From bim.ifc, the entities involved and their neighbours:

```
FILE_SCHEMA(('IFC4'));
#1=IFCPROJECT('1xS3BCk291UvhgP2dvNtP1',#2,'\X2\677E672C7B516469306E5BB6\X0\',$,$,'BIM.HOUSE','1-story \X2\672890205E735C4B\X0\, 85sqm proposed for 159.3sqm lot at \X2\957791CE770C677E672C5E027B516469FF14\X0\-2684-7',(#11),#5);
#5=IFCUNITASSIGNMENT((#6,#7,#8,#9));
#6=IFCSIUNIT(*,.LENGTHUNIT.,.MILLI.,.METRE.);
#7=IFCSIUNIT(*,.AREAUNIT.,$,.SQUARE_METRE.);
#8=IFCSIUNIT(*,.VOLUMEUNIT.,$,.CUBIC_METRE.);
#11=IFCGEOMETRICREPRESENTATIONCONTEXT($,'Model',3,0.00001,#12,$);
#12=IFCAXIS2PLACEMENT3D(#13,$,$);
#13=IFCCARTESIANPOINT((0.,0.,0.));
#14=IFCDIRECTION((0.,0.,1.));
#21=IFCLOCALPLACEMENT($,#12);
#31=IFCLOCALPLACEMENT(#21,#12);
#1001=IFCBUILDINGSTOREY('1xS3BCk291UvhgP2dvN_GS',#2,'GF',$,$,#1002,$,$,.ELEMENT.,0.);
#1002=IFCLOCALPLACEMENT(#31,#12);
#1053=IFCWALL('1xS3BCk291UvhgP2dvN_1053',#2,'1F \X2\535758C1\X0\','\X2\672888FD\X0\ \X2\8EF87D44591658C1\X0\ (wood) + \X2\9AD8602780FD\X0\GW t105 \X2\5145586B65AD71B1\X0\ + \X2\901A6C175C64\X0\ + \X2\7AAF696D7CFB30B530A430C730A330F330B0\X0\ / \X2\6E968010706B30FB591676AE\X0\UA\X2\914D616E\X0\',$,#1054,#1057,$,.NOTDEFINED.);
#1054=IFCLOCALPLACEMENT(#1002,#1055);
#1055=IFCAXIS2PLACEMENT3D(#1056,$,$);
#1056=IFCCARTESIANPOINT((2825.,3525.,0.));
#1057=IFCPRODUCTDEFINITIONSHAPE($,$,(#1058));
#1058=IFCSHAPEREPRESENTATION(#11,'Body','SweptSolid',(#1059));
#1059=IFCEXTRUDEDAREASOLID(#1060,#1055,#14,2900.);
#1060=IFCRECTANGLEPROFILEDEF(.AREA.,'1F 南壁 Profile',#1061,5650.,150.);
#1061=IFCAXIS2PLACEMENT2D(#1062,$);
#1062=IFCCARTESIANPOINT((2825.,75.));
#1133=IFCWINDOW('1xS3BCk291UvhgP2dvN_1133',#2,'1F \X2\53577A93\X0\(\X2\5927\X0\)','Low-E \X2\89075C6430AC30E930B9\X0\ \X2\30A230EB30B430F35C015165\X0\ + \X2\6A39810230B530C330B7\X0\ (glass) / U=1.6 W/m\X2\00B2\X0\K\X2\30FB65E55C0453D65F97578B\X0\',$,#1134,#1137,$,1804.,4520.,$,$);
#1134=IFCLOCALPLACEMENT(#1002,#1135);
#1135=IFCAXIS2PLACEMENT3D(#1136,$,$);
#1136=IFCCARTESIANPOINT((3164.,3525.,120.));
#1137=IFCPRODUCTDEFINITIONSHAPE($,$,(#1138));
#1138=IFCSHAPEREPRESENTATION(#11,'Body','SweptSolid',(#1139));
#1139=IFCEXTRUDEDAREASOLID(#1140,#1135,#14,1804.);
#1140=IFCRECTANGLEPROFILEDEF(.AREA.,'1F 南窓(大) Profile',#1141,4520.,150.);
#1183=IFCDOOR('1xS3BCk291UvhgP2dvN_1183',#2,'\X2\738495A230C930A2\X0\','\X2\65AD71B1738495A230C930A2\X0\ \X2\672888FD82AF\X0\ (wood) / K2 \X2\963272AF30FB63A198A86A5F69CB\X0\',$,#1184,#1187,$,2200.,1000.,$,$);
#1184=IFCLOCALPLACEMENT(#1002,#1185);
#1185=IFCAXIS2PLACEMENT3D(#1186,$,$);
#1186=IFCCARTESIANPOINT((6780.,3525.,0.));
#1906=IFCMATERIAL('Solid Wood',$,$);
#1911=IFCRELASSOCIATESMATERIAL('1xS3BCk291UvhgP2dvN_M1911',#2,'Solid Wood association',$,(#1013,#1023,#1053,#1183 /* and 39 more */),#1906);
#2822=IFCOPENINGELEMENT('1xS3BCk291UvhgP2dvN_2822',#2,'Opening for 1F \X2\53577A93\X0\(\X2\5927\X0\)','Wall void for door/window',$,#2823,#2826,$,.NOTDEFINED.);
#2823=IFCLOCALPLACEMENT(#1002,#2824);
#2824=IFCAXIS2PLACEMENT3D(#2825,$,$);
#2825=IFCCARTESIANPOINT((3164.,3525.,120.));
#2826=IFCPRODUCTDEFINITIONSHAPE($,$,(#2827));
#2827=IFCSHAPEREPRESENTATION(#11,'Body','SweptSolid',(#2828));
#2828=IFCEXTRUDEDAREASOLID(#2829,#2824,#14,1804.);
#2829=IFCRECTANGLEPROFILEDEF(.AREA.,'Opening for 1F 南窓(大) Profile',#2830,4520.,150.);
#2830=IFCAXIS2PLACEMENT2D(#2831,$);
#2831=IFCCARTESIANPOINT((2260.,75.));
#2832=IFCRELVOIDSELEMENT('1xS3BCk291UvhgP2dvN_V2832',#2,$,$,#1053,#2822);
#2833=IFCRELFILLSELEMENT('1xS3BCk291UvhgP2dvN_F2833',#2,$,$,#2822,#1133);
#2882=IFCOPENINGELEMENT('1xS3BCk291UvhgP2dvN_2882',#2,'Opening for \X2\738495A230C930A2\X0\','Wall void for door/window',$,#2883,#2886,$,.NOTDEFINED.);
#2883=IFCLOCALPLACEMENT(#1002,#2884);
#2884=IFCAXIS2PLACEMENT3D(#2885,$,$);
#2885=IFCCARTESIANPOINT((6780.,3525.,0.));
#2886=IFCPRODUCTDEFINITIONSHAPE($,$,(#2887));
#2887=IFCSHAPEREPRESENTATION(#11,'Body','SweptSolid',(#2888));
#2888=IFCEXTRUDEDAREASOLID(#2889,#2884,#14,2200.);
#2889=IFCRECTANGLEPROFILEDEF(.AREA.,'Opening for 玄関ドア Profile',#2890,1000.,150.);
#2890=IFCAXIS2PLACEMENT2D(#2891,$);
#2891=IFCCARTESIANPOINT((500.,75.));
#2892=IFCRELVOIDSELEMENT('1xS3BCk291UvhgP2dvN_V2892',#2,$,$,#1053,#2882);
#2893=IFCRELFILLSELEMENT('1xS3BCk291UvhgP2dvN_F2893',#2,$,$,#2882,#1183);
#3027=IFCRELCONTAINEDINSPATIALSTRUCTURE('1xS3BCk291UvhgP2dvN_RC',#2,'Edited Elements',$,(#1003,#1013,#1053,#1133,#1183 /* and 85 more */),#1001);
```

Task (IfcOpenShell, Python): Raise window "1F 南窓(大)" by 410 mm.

```python
import numpy as np
import ifcopenshell
import ifcopenshell.api.geometry
import ifcopenshell.util.placement
import ifcopenshell.util.unit

model = ifcopenshell.open("bim.ifc")
unit_scale = ifcopenshell.util.unit.calculate_unit_scale(model)

window = model.by_id(1133)
opening = window.FillsVoids[0].RelatingOpeningElement
dz = 0.41 / unit_scale

shift = np.array([0.0, 0.0, dz])
# The window is not placed relative to its opening, so move both.
for product in (opening, window):
    matrix = ifcopenshell.util.placement.get_local_placement(product.ObjectPlacement)
    matrix[:3, 3] += shift
    ifcopenshell.api.geometry.edit_object_placement(model, product=product, matrix=matrix, is_si=False)

print(f"moved by {dz * unit_scale:+.3f} m")

model.write("bim-out.ifc")
```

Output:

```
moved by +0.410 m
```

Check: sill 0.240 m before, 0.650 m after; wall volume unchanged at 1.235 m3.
